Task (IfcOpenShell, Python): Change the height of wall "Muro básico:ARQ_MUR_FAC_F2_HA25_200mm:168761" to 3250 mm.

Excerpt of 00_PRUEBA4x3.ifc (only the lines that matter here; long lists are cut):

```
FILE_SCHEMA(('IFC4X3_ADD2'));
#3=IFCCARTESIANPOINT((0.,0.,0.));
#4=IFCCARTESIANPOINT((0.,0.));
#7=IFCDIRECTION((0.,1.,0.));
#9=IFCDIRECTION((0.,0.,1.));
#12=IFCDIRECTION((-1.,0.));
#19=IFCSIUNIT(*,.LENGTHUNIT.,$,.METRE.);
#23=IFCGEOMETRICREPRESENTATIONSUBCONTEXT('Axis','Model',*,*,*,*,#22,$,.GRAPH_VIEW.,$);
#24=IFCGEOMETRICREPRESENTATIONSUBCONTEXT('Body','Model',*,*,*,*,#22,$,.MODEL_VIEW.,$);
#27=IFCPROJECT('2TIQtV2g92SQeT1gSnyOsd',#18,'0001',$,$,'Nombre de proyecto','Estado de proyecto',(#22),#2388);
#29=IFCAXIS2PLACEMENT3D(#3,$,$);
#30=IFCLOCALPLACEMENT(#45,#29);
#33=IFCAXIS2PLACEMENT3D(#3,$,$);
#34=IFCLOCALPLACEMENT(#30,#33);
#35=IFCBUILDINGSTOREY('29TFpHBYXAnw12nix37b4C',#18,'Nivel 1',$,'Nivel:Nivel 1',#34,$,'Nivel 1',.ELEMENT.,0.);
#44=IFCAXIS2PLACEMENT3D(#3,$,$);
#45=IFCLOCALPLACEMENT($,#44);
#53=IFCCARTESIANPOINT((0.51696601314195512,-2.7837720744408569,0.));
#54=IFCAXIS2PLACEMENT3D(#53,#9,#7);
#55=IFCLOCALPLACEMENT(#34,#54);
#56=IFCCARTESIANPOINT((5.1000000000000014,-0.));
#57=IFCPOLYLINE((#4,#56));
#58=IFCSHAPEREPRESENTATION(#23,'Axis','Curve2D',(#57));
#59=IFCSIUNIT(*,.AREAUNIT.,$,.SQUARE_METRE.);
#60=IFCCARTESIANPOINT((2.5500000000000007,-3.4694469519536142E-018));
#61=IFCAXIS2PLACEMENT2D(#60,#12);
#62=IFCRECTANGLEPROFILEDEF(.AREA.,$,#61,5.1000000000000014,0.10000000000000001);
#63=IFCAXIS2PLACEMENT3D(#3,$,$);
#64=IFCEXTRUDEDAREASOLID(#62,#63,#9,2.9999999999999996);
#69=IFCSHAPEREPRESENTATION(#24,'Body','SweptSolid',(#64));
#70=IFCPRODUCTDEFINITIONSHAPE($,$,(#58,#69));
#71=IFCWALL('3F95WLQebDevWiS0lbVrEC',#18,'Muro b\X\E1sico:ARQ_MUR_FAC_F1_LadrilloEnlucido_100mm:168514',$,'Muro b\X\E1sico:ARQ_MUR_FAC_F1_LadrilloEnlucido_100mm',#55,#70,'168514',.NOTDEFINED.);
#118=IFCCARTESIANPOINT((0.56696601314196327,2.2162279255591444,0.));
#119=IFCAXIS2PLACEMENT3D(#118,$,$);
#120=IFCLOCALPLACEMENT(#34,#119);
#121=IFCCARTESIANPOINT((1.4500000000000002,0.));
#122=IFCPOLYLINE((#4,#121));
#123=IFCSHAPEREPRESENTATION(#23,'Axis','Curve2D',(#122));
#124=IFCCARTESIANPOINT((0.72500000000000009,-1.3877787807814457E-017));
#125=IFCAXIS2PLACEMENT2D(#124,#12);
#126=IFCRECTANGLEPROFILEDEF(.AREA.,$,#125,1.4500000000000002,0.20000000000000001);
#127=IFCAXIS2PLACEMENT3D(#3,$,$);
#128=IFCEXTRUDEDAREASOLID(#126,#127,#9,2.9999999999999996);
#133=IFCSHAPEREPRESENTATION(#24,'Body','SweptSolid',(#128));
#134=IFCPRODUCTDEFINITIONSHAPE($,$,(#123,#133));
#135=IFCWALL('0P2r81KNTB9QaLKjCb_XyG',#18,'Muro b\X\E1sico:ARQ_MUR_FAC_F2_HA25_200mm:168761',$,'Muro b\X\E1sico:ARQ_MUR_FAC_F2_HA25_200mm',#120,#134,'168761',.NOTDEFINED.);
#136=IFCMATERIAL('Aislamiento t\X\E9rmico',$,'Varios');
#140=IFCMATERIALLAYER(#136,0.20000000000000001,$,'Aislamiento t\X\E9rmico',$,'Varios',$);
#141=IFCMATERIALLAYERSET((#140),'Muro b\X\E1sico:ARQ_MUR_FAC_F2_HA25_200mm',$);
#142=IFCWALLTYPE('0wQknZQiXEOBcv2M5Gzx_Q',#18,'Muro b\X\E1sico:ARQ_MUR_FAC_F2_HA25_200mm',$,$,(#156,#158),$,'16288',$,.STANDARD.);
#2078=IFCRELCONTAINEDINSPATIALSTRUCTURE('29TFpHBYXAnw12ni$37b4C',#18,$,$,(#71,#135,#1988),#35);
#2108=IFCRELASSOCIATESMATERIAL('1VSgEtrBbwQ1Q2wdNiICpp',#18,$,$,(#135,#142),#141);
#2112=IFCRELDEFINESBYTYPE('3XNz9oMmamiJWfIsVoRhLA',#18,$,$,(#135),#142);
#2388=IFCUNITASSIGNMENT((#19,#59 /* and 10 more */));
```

```python
import ifcopenshell
import ifcopenshell.geom
import ifcopenshell.util.representation
import ifcopenshell.util.shape
import ifcopenshell.util.unit

model = ifcopenshell.open("00_PRUEBA4x3.ifc")
unit_scale = ifcopenshell.util.unit.calculate_unit_scale(model)
settings = ifcopenshell.geom.settings()


def volume(element):
    """Net volume in cubic metres, openings subtracted."""
    shape = ifcopenshell.geom.create_shape(settings, element)
    return ifcopenshell.util.shape.get_volume(shape.geometry)


wall = model.by_guid("0P2r81KNTB9QaLKjCb_XyG")
before = volume(wall)

body = ifcopenshell.util.representation.get_representation(wall, "Model", "Body")
solid = body.Items[0]
old_height = solid.Depth
solid.Depth = 3.25 / unit_scale
after = volume(wall)

print(f"height {old_height:g} -> {solid.Depth:g}, volume {before:.3f} -> {after:.3f} m3")

model.write("00_PRUEBA4x3_updated.ifc")
```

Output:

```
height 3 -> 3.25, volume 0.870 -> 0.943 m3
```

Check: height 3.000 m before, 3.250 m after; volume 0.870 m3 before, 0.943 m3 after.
